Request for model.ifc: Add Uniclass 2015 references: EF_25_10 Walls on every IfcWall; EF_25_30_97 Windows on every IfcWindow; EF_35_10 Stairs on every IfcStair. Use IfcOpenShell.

First a look at what the model holds.

```python
import ifcopenshell

model = ifcopenshell.open("model.ifc")
print(model.schema)
print("classifications:", [c.Name for c in model.by_type("IfcClassification")])
for ifc_class in ("IfcDoor", "IfcRoof", "IfcStair", "IfcWall", "IfcWindow"):
    print(ifc_class, len(model.by_type(ifc_class)))
```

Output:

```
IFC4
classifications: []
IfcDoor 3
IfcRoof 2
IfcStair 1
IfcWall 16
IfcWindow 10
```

```python
import ifcopenshell
import ifcopenshell.api.classification

model = ifcopenshell.open("model.ifc")

system = ifcopenshell.api.classification.add_classification(model, classification="Uniclass 2015")

codes = {
    "IfcWall": ("EF_25_10", "Walls"),
    "IfcWindow": ("EF_25_30_97", "Windows"),
    "IfcStair": ("EF_35_10", "Stairs"),
}
for ifc_class, (code, name) in codes.items():
    products = model.by_type(ifc_class)
    ifcopenshell.api.classification.add_reference(
        model, products=products, classification=system, identification=code, name=name
    )
    print(code, len(products))

model.write("model-out.ifc")
```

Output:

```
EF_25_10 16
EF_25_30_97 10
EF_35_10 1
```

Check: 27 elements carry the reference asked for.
